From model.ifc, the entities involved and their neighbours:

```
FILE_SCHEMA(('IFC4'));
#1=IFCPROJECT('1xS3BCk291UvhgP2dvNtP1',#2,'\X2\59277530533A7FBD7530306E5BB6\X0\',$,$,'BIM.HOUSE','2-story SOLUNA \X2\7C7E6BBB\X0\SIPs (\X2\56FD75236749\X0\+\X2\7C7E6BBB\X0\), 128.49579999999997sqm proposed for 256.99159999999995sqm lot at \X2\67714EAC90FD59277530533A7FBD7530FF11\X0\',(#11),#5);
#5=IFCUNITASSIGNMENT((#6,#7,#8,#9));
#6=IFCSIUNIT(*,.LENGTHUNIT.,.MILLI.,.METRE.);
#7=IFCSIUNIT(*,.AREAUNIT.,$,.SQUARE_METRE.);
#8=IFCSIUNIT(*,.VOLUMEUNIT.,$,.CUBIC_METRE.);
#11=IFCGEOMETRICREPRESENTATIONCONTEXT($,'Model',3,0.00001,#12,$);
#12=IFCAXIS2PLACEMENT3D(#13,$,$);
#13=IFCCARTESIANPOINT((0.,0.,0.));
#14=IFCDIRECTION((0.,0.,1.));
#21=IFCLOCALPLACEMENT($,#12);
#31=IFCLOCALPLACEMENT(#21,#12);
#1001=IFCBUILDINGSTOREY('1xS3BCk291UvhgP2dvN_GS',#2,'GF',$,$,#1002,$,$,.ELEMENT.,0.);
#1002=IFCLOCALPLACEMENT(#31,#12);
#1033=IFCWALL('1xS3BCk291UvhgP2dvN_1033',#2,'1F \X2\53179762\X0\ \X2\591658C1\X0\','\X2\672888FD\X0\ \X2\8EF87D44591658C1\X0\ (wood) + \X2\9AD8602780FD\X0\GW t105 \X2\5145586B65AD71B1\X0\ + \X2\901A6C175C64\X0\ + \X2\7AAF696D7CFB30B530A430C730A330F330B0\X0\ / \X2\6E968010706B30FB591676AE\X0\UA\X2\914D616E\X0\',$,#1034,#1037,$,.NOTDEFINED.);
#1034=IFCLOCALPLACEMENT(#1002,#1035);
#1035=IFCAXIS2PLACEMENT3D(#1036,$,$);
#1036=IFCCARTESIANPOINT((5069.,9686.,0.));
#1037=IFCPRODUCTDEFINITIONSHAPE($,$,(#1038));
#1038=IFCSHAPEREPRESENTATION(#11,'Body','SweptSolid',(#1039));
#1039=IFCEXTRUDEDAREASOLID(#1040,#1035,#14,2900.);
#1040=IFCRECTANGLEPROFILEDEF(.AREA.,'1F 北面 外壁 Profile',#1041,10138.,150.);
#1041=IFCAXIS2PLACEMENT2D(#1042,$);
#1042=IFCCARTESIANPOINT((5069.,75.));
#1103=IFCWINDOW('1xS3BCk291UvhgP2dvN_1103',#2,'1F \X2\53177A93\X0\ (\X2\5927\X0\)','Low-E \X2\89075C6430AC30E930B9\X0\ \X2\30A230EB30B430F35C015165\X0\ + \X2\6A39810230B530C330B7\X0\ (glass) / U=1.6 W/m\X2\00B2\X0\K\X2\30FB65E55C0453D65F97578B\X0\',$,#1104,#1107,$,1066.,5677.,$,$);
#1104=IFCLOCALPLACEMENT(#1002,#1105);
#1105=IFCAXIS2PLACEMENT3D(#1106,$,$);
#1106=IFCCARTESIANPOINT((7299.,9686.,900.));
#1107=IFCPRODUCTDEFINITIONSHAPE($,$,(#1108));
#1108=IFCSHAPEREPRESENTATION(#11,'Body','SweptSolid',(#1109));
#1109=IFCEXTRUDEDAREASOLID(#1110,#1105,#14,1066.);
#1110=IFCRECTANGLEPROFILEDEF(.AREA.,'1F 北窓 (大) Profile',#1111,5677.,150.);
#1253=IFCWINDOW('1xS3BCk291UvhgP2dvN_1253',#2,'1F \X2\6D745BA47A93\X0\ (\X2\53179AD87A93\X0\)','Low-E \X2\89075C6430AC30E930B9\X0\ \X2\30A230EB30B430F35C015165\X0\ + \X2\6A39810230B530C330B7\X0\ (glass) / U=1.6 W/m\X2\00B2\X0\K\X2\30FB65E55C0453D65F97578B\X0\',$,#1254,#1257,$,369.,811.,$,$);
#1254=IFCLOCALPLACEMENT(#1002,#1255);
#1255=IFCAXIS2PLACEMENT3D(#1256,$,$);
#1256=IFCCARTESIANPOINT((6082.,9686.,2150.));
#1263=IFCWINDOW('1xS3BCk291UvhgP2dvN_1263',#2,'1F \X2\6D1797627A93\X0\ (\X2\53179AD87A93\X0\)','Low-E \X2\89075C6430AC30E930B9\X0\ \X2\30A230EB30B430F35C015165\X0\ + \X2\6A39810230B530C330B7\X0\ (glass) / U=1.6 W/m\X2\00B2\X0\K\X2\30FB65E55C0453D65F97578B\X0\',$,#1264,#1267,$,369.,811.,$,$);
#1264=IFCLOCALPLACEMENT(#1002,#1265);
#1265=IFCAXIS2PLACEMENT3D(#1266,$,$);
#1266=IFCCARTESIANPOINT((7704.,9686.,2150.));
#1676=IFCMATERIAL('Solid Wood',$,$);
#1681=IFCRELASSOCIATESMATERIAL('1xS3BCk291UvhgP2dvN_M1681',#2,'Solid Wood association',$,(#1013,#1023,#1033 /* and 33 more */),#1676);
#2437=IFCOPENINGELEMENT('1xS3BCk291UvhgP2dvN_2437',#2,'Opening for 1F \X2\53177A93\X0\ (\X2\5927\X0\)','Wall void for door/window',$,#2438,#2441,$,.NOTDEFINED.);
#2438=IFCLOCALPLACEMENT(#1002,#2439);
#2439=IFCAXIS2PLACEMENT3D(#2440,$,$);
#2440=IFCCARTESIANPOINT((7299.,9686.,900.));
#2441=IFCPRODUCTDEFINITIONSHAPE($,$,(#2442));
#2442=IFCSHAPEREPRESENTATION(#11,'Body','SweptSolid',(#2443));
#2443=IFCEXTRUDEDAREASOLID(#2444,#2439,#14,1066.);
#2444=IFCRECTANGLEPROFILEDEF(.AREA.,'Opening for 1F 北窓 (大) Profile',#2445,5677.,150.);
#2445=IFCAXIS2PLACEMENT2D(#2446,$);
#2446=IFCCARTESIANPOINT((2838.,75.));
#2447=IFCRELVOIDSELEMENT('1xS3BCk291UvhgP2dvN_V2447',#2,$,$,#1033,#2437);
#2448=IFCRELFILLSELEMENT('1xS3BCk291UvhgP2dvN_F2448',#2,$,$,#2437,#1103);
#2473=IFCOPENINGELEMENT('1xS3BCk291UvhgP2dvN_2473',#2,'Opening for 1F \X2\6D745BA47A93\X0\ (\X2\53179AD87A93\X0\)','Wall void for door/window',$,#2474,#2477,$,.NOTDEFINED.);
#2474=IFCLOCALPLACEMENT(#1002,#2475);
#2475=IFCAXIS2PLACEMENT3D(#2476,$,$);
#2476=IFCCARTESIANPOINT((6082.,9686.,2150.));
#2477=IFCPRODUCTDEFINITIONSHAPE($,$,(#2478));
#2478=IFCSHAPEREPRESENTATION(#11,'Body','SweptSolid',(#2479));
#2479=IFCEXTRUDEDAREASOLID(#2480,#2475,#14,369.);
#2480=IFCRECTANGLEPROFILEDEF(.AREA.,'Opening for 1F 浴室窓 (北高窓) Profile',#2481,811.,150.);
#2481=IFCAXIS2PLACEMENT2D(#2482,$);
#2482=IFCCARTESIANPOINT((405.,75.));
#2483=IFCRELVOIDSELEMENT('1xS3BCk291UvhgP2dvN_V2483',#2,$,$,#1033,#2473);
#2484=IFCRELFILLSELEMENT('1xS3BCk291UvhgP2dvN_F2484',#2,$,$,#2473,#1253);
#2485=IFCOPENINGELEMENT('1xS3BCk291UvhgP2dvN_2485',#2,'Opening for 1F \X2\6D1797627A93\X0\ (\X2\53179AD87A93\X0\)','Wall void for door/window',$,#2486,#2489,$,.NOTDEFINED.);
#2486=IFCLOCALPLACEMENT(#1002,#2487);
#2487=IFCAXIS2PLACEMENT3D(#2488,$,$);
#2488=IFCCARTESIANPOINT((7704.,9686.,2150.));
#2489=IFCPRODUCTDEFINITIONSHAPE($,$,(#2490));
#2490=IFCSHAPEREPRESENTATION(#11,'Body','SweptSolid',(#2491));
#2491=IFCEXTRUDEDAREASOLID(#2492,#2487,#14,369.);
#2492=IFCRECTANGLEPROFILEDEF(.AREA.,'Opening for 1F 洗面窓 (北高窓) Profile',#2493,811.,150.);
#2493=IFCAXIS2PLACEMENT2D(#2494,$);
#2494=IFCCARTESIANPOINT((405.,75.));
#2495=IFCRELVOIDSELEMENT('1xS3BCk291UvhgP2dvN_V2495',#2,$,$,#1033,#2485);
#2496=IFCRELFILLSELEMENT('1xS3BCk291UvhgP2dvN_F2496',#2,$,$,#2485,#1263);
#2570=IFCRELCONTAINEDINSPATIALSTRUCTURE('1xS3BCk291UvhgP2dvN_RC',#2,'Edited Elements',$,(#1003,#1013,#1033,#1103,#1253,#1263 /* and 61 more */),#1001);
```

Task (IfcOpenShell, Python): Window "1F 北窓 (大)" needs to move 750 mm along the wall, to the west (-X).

```python
import ifcopenshell
import ifcopenshell.api.geometry
import ifcopenshell.util.placement

model = ifcopenshell.open("model.ifc")

window = model.by_guid("1xS3BCk291UvhgP2dvN_1103")
opening = window.FillsVoids[0].RelatingOpeningElement
wall = opening.VoidsElements[0].RelatingBuildingElement

wall_matrix = ifcopenshell.util.placement.get_local_placement(wall.ObjectPlacement)
shift = wall_matrix[:3, 0] * -750.0
before = ifcopenshell.util.placement.get_local_placement(window.ObjectPlacement)[:3, 3].copy()

# The window is not placed relative to its opening, so move both.
for product in (opening, window):
    matrix = ifcopenshell.util.placement.get_local_placement(product.ObjectPlacement)
    matrix[:3, 3] += shift
    ifcopenshell.api.geometry.edit_object_placement(model, product=product, matrix=matrix, is_si=False)

after = ifcopenshell.util.placement.get_local_placement(window.ObjectPlacement)[:3, 3]
print("window moved by", (after - before).round(3) + 0.0)

model.write("model_v2.ifc")
```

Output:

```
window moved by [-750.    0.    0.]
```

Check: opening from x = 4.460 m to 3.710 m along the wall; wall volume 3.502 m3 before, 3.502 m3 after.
